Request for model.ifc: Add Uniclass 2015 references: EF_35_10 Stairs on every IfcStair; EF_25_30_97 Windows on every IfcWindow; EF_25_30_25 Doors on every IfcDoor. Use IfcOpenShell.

First a look at what the model holds.

```python
import ifcopenshell

model = ifcopenshell.open("model.ifc")
print(model.schema)
print("classifications:", [c.Name for c in model.by_type("IfcClassification")])
for ifc_class in ("IfcDoor", "IfcRoof", "IfcStair", "IfcWall", "IfcWindow"):
    print(ifc_class, len(model.by_type(ifc_class)))
```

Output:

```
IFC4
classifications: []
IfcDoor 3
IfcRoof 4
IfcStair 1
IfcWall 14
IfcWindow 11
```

```python
import ifcopenshell
import ifcopenshell.api.classification

model = ifcopenshell.open("model.ifc")

system = ifcopenshell.api.classification.add_classification(model, classification="Uniclass 2015")

codes = {
    "IfcStair": ("EF_35_10", "Stairs"),
    "IfcWindow": ("EF_25_30_97", "Windows"),
    "IfcDoor": ("EF_25_30_25", "Doors"),
}
for ifc_class, (code, name) in codes.items():
    products = model.by_type(ifc_class)
    ifcopenshell.api.classification.add_reference(
        model, products=products, classification=system, identification=code, name=name
    )
    print(code, len(products))

model.write("model_rev.ifc")
```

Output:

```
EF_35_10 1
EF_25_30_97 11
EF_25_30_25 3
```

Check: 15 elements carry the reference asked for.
